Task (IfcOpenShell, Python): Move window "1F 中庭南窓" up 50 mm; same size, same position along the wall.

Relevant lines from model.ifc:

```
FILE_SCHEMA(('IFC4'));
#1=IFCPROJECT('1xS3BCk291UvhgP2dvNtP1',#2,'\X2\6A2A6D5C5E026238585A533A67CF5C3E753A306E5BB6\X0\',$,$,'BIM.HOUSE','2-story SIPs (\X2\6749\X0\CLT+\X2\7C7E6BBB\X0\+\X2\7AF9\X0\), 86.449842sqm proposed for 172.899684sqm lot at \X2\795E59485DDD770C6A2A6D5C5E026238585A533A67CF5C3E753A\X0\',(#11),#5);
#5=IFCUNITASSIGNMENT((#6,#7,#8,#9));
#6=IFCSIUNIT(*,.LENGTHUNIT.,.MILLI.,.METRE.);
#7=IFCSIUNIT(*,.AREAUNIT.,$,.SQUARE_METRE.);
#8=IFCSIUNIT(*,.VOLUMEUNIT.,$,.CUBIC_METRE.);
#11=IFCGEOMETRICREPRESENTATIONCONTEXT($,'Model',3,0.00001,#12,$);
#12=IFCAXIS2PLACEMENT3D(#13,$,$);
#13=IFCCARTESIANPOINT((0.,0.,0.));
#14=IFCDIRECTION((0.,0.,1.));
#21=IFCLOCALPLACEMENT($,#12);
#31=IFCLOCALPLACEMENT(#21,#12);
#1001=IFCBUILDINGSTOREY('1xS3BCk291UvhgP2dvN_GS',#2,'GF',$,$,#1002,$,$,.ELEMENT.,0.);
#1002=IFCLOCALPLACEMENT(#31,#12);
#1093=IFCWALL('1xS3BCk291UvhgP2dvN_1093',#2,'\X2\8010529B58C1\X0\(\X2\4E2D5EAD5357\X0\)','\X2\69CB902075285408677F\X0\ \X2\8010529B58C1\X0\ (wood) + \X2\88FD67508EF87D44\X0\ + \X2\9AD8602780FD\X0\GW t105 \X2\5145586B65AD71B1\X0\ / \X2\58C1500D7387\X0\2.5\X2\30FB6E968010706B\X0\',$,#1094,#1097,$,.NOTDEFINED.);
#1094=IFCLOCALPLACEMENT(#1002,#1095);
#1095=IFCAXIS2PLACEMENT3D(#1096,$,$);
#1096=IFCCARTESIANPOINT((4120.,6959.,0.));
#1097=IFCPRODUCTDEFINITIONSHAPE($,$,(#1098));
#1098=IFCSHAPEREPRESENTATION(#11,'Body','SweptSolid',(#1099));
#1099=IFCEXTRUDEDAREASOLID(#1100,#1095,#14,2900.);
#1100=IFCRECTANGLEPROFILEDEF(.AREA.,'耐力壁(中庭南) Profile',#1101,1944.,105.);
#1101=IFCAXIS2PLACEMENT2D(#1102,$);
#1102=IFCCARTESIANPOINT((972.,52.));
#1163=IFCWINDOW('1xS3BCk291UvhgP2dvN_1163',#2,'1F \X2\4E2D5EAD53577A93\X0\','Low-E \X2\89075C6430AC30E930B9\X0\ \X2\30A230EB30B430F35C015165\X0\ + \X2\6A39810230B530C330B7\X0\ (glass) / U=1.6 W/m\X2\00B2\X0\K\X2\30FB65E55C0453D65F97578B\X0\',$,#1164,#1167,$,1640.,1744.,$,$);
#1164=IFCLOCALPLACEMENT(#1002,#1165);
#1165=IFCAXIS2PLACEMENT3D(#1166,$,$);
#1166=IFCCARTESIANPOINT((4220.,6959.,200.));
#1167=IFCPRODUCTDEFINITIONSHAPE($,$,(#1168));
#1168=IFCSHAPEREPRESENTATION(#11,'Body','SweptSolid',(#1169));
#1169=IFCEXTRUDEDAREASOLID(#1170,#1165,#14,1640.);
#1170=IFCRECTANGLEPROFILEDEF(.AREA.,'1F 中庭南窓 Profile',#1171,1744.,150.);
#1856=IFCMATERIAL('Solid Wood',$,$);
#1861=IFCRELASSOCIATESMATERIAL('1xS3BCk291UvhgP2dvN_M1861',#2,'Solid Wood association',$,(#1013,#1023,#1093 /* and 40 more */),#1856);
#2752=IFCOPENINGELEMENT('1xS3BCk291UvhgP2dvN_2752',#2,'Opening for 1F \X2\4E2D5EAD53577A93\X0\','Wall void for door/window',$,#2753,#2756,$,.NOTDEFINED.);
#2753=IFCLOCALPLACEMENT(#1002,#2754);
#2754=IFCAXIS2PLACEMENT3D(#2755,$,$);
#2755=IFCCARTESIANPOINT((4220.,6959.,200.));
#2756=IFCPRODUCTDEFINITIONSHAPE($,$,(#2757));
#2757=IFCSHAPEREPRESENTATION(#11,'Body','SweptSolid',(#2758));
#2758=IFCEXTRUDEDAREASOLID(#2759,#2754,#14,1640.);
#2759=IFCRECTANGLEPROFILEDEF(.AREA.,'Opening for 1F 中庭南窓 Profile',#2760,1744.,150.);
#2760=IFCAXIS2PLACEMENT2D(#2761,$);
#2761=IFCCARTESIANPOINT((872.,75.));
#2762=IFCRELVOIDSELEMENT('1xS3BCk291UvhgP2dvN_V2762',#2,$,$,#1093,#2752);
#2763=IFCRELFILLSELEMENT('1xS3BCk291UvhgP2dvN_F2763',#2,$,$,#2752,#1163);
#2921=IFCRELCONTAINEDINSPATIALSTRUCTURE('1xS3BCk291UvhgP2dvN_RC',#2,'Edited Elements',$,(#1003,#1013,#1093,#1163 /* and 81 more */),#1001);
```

```python
import numpy as np
import ifcopenshell
import ifcopenshell.api.geometry
import ifcopenshell.util.placement
import ifcopenshell.util.unit

model = ifcopenshell.open("model.ifc")
unit_scale = ifcopenshell.util.unit.calculate_unit_scale(model)

window = model.by_guid("1xS3BCk291UvhgP2dvN_1163")
opening = window.FillsVoids[0].RelatingOpeningElement
dz = 0.05 / unit_scale

shift = np.array([0.0, 0.0, dz])
# The window is not placed relative to its opening, so move both.
for product in (opening, window):
    matrix = ifcopenshell.util.placement.get_local_placement(product.ObjectPlacement)
    matrix[:3, 3] += shift
    ifcopenshell.api.geometry.edit_object_placement(model, product=product, matrix=matrix, is_si=False)

print(f"moved by {dz * unit_scale:+.3f} m")

model.write("model_v2.ifc")
```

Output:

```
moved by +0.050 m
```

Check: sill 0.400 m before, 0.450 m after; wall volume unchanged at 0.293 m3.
